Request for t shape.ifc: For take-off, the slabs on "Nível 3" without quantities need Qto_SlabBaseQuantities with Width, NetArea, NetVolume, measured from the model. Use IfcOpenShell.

First a look at what the model holds.

```python
import ifcopenshell
import ifcopenshell.util.element
import ifcopenshell.util.unit

model = ifcopenshell.open("t shape.ifc")
print(model.schema)
for unit_type in ("LENGTHUNIT", "AREAUNIT", "VOLUMEUNIT"):
    print(unit_type, ifcopenshell.util.unit.calculate_unit_scale(model, unit_type))
storey = next(s for s in model.by_type("IfcBuildingStorey") if s.Name == "Nível 3")
slabs = [e for e in ifcopenshell.util.element.get_decomposition(storey) if e.is_a("IfcSlab")]
for e in sorted(slabs, key=lambda e: e.id()):
    print(e.id(), e.is_a(), e.Name, list(ifcopenshell.util.element.get_psets(e, qtos_only=True)), sep=" | ")
```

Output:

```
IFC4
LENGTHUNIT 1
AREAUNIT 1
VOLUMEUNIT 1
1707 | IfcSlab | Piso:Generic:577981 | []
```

```python
import ifcopenshell
import ifcopenshell.api.pset
import ifcopenshell.geom
import ifcopenshell.util.element
import ifcopenshell.util.shape
import ifcopenshell.util.unit

model = ifcopenshell.open("t shape.ifc")
unit_scale = ifcopenshell.util.unit.calculate_unit_scale(model)
area_scale = ifcopenshell.util.unit.calculate_unit_scale(model, "AREAUNIT")
volume_scale = ifcopenshell.util.unit.calculate_unit_scale(model, "VOLUMEUNIT")
settings = ifcopenshell.geom.settings()

storey = next(s for s in model.by_type("IfcBuildingStorey") if s.Name == "Nível 3")
slabs = [e for e in ifcopenshell.util.element.get_decomposition(storey) if e.is_a("IfcSlab")]

for e in sorted(slabs, key=lambda e: e.id()):
    if ifcopenshell.util.element.get_psets(e, qtos_only=True, should_inherit=False):
        continue
    # Geometry comes back in metres, in the element's own axes.
    shape = ifcopenshell.geom.create_shape(settings, e)
    values = {
        "Width": ifcopenshell.util.shape.get_z(shape.geometry) / unit_scale,
        "NetArea": ifcopenshell.util.shape.get_footprint_area(shape.geometry) / area_scale,
        "NetVolume": ifcopenshell.util.shape.get_volume(shape.geometry) / volume_scale,
    }
    qto = ifcopenshell.api.pset.add_qto(model, product=e, name="Qto_SlabBaseQuantities")
    ifcopenshell.api.pset.edit_qto(model, qto=qto, properties=values)
    print(e.id(), {k: round(v, 3) for k, v in values.items()})

model.write("t shape_v2.ifc")
```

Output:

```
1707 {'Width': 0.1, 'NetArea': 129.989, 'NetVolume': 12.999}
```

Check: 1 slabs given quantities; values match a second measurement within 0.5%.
